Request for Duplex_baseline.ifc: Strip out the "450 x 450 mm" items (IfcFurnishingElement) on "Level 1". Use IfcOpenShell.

First a look at what the model holds.

```python
import ifcopenshell
import ifcopenshell.util.element

model = ifcopenshell.open("Duplex_baseline.ifc")
print(model.schema)
storey = next(s for s in model.by_type("IfcBuildingStorey") if s.Name == "Level 1")
furniture = [e for e in ifcopenshell.util.element.get_decomposition(storey) if e.is_a("IfcFurnishingElement")]
seen = {}
for e in furniture:
    element_type = ifcopenshell.util.element.get_type(e)
    name = element_type.Name if element_type not in (None, e) else None
    seen[name] = seen.get(name, 0) + 1
for name, count in sorted(seen.items(), key=str):
    print(count, "x", name)
```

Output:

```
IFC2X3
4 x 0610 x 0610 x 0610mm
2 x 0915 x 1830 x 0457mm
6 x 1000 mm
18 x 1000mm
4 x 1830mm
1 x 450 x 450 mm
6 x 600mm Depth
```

```python
import ifcopenshell
import ifcopenshell.api.root
import ifcopenshell.util.element

model = ifcopenshell.open("Duplex_baseline.ifc")

storey = next(s for s in model.by_type("IfcBuildingStorey") if s.Name == "Level 1")
furniture = [e for e in ifcopenshell.util.element.get_decomposition(storey) if e.is_a("IfcFurnishingElement")]
targets = [e for e in furniture if (t := ifcopenshell.util.element.get_type(e)) not in (None, e) and t.Name == "450 x 450 mm"]

for e in targets:
    ifcopenshell.api.root.remove_product(model, product=e)
print(len(targets), "removed")

model.write("Duplex_baseline-out.ifc")
```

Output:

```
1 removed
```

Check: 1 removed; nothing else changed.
